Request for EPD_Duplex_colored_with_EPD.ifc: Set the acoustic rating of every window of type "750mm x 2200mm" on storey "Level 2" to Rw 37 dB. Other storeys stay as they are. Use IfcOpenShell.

First a look at what the model holds.

```python
import ifcopenshell
import ifcopenshell.util.element

model = ifcopenshell.open("EPD_Duplex_colored_with_EPD.ifc")
print(model.schema)
storey = next(s for s in model.by_type("IfcBuildingStorey") if s.Name == "Level 2")
windows = [e for e in ifcopenshell.util.element.get_decomposition(storey) if e.is_a("IfcWindow")]
seen = {}
for e in windows:
    element_type = ifcopenshell.util.element.get_type(e)
    key = (element_type.Name if element_type != e and element_type else None, ifcopenshell.util.element.get_pset(e, "Pset_WindowCommon", "AcousticRating"))
    seen[key] = seen.get(key, 0) + 1
for (name, value), count in sorted(seen.items(), key=str):
    print(count, "x", name, "|", value)
```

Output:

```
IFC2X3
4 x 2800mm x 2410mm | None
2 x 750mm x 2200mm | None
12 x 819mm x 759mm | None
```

```python
import ifcopenshell
import ifcopenshell.api.pset
import ifcopenshell.util.element

model = ifcopenshell.open("EPD_Duplex_colored_with_EPD.ifc")

storey = next(s for s in model.by_type("IfcBuildingStorey") if s.Name == "Level 2")
windows = [e for e in ifcopenshell.util.element.get_decomposition(storey) if e.is_a("IfcWindow")]

count = 0
for e in windows:
    element_type = ifcopenshell.util.element.get_type(e)
    if element_type in (None, e) or element_type.Name != "750mm x 2200mm":
        continue
    # add_pset returns the element's existing set when there is one.
    pset = ifcopenshell.api.pset.add_pset(model, product=e, name="Pset_WindowCommon")
    ifcopenshell.api.pset.edit_pset(model, pset=pset, properties={"AcousticRating": "Rw 37 dB"})
    count += 1

print(count, "windows updated")

model.write("EPD_Duplex_colored_with_EPD_v2.ifc")
```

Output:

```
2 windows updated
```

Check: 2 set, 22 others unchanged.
